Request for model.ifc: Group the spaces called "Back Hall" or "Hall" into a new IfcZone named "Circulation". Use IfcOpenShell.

First a look at what the model holds.

```python
import ifcopenshell

model = ifcopenshell.open("model.ifc")
print(model.schema)
seen = {}
for space in model.by_type("IfcSpace"):
    seen[space.LongName] = seen.get(space.LongName, 0) + 1
for name, count in sorted(seen.items(), key=str):
    print(count, "x", name)
print("zones:", [z.Name for z in model.by_type("IfcZone")][:20])
```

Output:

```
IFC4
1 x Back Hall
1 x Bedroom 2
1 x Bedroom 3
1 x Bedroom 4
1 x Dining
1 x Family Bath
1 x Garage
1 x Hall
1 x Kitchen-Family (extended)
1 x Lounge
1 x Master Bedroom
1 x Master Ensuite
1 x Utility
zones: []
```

```python
import ifcopenshell
import ifcopenshell.api.group
import ifcopenshell.api.root

model = ifcopenshell.open("model.ifc")

names = {"Back Hall", "Hall"}
spaces = [s for s in model.by_type("IfcSpace") if s.LongName in names]

zone = ifcopenshell.api.root.create_entity(model, ifc_class="IfcZone", name="Circulation")
ifcopenshell.api.group.assign_group(model, products=spaces, group=zone)
print(len(spaces), "spaces in", zone.Name)

model.write("model_edited.ifc")
```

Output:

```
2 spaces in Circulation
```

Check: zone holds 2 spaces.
